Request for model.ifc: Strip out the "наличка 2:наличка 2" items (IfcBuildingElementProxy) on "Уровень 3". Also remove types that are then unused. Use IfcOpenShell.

First a look at what the model holds.

```python
import ifcopenshell
import ifcopenshell.util.element

model = ifcopenshell.open("model.ifc")
print(model.schema)
storey = next(s for s in model.by_type("IfcBuildingStorey") if s.Name == "Уровень 3")
proxies = [e for e in ifcopenshell.util.element.get_decomposition(storey) if e.is_a("IfcBuildingElementProxy")]
seen = {}
for e in proxies:
    element_type = ifcopenshell.util.element.get_type(e)
    name = element_type.Name if element_type not in (None, e) else None
    seen[name] = seen.get(name, 0) + 1
for name, count in sorted(seen.items(), key=str):
    print(count, "x", name)
```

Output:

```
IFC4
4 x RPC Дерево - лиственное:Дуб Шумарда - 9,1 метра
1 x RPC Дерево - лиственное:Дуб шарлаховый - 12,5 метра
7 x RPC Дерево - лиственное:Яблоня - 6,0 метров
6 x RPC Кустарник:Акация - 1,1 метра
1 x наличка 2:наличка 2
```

```python
import ifcopenshell
import ifcopenshell.api.root
import ifcopenshell.util.element

model = ifcopenshell.open("model.ifc")

storey = next(s for s in model.by_type("IfcBuildingStorey") if s.Name == "Уровень 3")
proxies = [e for e in ifcopenshell.util.element.get_decomposition(storey) if e.is_a("IfcBuildingElementProxy")]
targets = [e for e in proxies if (t := ifcopenshell.util.element.get_type(e)) not in (None, e) and t.Name == "наличка 2:наличка 2"]
types = {ifcopenshell.util.element.get_type(e) for e in targets} - {None, *targets}

for e in targets:
    ifcopenshell.api.root.remove_product(model, product=e)
print(len(targets), "removed")

unused = [t for t in types if not ifcopenshell.util.element.get_types(t)]
for t in unused:
    ifcopenshell.api.root.remove_product(model, product=t)
print(len(unused), "unused types removed")

model.write("model-out.ifc")
```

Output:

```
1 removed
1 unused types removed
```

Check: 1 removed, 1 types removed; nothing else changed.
